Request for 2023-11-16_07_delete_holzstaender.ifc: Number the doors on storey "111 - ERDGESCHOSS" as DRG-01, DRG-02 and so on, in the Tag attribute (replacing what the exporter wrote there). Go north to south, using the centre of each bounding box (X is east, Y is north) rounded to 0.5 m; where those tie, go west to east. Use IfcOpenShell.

First a look at what the model holds.

```python
import ifcopenshell
import ifcopenshell.util.element
import ifcopenshell.util.placement

model = ifcopenshell.open("2023-11-16_07_delete_holzstaender.ifc")
print(model.schema)
storey = next(s for s in model.by_type("IfcBuildingStorey") if s.Name == "111 - ERDGESCHOSS")
doors = [e for e in ifcopenshell.util.element.get_decomposition(storey) if e.is_a("IfcDoor")]
for e in sorted(doors, key=lambda e: e.id()):
    origin = ifcopenshell.util.placement.get_local_placement(e.ObjectPlacement)[:3, 3]
    print(e.id(), e.Tag, e.Name, origin.round(2) + 0.0, sep=" | ")
```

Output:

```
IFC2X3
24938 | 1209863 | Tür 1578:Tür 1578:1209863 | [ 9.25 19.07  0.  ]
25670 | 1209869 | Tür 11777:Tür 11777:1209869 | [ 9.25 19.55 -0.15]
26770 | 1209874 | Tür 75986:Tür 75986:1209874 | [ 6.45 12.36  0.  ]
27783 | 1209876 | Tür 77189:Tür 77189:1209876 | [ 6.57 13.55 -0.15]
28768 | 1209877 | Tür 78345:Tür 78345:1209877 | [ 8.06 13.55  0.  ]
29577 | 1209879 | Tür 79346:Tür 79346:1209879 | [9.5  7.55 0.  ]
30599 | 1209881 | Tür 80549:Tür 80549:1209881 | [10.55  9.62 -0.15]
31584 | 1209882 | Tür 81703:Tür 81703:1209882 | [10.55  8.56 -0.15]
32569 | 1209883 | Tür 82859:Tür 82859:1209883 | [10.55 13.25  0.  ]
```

```python
import ifcopenshell
import ifcopenshell.geom
import ifcopenshell.util.element
import ifcopenshell.util.shape

model = ifcopenshell.open("2023-11-16_07_delete_holzstaender.ifc")
settings = ifcopenshell.geom.settings()
settings.set("use-world-coords", True)


def centre(element):
    shape = ifcopenshell.geom.create_shape(settings, element)
    return ifcopenshell.util.shape.get_bbox_centroid(shape.geometry)


storey = next(s for s in model.by_type("IfcBuildingStorey") if s.Name == "111 - ERDGESCHOSS")
doors = [e for e in ifcopenshell.util.element.get_decomposition(storey) if e.is_a("IfcDoor")]

# Insertion points can sit at a corner or the storey origin, so sort by the geometry (in metres).
centres = {e: centre(e) for e in doors}
doors.sort(key=lambda e: (-round(centres[e][1] / 0.5), centres[e][0]))

for i, e in enumerate(doors, start=1):
    number = f"DRG-{i:02d}"
    e.Tag = number
    print(e.id(), number)

model.write("2023-11-16_07_delete_holzstaender_edited.ifc")
```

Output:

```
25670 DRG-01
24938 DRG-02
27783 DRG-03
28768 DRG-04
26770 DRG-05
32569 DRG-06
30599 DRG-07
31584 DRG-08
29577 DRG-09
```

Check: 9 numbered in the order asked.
